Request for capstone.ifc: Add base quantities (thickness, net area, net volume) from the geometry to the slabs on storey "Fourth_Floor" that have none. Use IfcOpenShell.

First a look at what the model holds.

```python
import ifcopenshell
import ifcopenshell.util.element
import ifcopenshell.util.unit

model = ifcopenshell.open("capstone.ifc")
print(model.schema)
for unit_type in ("LENGTHUNIT", "AREAUNIT", "VOLUMEUNIT"):
    print(unit_type, ifcopenshell.util.unit.calculate_unit_scale(model, unit_type))
storey = next(s for s in model.by_type("IfcBuildingStorey") if s.Name == "Fourth_Floor")
slabs = [e for e in ifcopenshell.util.element.get_decomposition(storey) if e.is_a("IfcSlab")]
for e in sorted(slabs, key=lambda e: e.id()):
    print(e.id(), e.is_a(), e.Name, list(ifcopenshell.util.element.get_psets(e, qtos_only=True)), sep=" | ")
```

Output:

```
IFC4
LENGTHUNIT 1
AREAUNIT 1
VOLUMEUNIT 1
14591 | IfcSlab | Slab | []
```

```python
import ifcopenshell
import ifcopenshell.api.pset
import ifcopenshell.geom
import ifcopenshell.util.element
import ifcopenshell.util.shape
import ifcopenshell.util.unit

model = ifcopenshell.open("capstone.ifc")
unit_scale = ifcopenshell.util.unit.calculate_unit_scale(model)
area_scale = ifcopenshell.util.unit.calculate_unit_scale(model, "AREAUNIT")
volume_scale = ifcopenshell.util.unit.calculate_unit_scale(model, "VOLUMEUNIT")
settings = ifcopenshell.geom.settings()

storey = next(s for s in model.by_type("IfcBuildingStorey") if s.Name == "Fourth_Floor")
slabs = [e for e in ifcopenshell.util.element.get_decomposition(storey) if e.is_a("IfcSlab")]

for e in sorted(slabs, key=lambda e: e.id()):
    if ifcopenshell.util.element.get_psets(e, qtos_only=True, should_inherit=False):
        continue
    # Geometry comes back in metres, in the element's own axes.
    shape = ifcopenshell.geom.create_shape(settings, e)
    values = {
        "Width": ifcopenshell.util.shape.get_z(shape.geometry) / unit_scale,
        "NetArea": ifcopenshell.util.shape.get_footprint_area(shape.geometry) / area_scale,
        "NetVolume": ifcopenshell.util.shape.get_volume(shape.geometry) / volume_scale,
    }
    qto = ifcopenshell.api.pset.add_qto(model, product=e, name="Qto_SlabBaseQuantities")
    ifcopenshell.api.pset.edit_qto(model, qto=qto, properties=values)
    print(e.id(), {k: round(v, 3) for k, v in values.items()})

model.write("capstone_edited.ifc")
```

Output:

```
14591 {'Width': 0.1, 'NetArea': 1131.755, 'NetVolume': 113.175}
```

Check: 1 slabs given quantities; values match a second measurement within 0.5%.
